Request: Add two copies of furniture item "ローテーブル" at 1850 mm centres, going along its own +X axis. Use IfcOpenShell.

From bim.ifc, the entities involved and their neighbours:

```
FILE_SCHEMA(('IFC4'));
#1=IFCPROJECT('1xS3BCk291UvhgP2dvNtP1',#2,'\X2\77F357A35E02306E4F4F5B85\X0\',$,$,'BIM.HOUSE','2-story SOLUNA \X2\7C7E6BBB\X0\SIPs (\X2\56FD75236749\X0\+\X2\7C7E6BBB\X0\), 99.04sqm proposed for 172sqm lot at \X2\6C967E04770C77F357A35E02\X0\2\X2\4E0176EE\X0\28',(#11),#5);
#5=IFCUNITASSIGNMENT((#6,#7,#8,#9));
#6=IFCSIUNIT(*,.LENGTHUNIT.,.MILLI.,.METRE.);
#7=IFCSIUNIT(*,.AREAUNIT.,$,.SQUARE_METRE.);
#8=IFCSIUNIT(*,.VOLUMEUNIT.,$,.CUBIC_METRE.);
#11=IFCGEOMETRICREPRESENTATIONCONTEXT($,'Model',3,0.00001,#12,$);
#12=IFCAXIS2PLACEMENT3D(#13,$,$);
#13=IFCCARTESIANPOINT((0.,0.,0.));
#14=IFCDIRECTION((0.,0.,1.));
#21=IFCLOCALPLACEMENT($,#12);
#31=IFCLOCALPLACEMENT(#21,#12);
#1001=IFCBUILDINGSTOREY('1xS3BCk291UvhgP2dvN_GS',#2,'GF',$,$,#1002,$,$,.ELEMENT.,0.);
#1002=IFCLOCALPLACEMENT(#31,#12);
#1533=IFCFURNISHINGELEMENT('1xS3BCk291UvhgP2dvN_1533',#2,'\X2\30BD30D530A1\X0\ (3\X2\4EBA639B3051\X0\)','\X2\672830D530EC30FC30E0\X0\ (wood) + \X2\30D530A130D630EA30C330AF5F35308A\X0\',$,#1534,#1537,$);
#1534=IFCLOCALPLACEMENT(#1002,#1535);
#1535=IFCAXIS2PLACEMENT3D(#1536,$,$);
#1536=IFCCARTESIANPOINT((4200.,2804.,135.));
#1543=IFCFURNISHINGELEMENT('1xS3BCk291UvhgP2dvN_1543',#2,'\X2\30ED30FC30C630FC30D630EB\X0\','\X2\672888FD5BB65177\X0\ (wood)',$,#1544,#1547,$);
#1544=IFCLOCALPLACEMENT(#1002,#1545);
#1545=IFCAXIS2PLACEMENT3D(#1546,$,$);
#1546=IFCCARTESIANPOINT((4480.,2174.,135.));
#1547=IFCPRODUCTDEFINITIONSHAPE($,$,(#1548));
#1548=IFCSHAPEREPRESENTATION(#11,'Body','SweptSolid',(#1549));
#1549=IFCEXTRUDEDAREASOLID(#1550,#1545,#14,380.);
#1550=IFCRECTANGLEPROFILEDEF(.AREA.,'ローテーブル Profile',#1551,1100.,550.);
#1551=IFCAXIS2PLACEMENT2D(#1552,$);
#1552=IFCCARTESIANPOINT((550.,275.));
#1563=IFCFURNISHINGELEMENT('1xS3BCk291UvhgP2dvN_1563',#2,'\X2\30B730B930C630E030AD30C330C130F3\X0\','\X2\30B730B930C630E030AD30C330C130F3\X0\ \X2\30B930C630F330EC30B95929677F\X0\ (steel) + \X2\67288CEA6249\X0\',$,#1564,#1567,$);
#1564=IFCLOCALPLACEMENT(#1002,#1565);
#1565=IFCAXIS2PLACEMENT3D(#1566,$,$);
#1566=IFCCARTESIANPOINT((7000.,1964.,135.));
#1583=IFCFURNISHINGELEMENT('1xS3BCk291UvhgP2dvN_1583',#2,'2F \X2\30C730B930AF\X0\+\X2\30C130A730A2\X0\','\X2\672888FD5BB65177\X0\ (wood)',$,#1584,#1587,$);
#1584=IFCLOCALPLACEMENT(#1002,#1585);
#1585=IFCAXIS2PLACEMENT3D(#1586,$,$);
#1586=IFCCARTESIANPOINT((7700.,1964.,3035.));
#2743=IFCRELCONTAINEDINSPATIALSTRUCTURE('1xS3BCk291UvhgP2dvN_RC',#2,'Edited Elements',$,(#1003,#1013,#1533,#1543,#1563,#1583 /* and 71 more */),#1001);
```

```python
import ifcopenshell
import ifcopenshell.api.geometry
import ifcopenshell.api.root
import ifcopenshell.util.element
import ifcopenshell.util.placement

model = ifcopenshell.open("bim.ifc")


def reuse_history(source, copy):
    """copy_class also copies each property set's owner history, people and application; keep the originals."""
    for rel in copy.IsDefinedBy:
        if rel.is_a("IfcRelDefinesByProperties") and (history := rel.RelatingPropertyDefinition.OwnerHistory):
            rel.RelatingPropertyDefinition.OwnerHistory = source.OwnerHistory
            ifcopenshell.util.element.remove_deep2(model, history)


source = model.by_guid("1xS3BCk291UvhgP2dvN_1543")
base = ifcopenshell.util.placement.get_local_placement(source.ObjectPlacement)
step = base[:3, 0] * 1850.0

for i in range(1, 3):
    copy = ifcopenshell.api.root.copy_class(model, product=source)
    copy.Representation = ifcopenshell.util.element.copy_deep(
        model, source.Representation, exclude=["IfcGeometricRepresentationContext", "IfcRepresentationMap"]
    )
    reuse_history(source, copy)
    matrix = base.copy()
    matrix[:3, 3] += i * step
    print("added at", matrix[:3, 3].round(3) + 0.0)
    ifcopenshell.api.geometry.edit_object_placement(model, product=copy, matrix=matrix, is_si=False)

model.write("bim_updated.ifc")
```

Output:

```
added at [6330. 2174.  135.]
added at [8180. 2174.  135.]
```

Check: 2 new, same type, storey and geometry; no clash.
